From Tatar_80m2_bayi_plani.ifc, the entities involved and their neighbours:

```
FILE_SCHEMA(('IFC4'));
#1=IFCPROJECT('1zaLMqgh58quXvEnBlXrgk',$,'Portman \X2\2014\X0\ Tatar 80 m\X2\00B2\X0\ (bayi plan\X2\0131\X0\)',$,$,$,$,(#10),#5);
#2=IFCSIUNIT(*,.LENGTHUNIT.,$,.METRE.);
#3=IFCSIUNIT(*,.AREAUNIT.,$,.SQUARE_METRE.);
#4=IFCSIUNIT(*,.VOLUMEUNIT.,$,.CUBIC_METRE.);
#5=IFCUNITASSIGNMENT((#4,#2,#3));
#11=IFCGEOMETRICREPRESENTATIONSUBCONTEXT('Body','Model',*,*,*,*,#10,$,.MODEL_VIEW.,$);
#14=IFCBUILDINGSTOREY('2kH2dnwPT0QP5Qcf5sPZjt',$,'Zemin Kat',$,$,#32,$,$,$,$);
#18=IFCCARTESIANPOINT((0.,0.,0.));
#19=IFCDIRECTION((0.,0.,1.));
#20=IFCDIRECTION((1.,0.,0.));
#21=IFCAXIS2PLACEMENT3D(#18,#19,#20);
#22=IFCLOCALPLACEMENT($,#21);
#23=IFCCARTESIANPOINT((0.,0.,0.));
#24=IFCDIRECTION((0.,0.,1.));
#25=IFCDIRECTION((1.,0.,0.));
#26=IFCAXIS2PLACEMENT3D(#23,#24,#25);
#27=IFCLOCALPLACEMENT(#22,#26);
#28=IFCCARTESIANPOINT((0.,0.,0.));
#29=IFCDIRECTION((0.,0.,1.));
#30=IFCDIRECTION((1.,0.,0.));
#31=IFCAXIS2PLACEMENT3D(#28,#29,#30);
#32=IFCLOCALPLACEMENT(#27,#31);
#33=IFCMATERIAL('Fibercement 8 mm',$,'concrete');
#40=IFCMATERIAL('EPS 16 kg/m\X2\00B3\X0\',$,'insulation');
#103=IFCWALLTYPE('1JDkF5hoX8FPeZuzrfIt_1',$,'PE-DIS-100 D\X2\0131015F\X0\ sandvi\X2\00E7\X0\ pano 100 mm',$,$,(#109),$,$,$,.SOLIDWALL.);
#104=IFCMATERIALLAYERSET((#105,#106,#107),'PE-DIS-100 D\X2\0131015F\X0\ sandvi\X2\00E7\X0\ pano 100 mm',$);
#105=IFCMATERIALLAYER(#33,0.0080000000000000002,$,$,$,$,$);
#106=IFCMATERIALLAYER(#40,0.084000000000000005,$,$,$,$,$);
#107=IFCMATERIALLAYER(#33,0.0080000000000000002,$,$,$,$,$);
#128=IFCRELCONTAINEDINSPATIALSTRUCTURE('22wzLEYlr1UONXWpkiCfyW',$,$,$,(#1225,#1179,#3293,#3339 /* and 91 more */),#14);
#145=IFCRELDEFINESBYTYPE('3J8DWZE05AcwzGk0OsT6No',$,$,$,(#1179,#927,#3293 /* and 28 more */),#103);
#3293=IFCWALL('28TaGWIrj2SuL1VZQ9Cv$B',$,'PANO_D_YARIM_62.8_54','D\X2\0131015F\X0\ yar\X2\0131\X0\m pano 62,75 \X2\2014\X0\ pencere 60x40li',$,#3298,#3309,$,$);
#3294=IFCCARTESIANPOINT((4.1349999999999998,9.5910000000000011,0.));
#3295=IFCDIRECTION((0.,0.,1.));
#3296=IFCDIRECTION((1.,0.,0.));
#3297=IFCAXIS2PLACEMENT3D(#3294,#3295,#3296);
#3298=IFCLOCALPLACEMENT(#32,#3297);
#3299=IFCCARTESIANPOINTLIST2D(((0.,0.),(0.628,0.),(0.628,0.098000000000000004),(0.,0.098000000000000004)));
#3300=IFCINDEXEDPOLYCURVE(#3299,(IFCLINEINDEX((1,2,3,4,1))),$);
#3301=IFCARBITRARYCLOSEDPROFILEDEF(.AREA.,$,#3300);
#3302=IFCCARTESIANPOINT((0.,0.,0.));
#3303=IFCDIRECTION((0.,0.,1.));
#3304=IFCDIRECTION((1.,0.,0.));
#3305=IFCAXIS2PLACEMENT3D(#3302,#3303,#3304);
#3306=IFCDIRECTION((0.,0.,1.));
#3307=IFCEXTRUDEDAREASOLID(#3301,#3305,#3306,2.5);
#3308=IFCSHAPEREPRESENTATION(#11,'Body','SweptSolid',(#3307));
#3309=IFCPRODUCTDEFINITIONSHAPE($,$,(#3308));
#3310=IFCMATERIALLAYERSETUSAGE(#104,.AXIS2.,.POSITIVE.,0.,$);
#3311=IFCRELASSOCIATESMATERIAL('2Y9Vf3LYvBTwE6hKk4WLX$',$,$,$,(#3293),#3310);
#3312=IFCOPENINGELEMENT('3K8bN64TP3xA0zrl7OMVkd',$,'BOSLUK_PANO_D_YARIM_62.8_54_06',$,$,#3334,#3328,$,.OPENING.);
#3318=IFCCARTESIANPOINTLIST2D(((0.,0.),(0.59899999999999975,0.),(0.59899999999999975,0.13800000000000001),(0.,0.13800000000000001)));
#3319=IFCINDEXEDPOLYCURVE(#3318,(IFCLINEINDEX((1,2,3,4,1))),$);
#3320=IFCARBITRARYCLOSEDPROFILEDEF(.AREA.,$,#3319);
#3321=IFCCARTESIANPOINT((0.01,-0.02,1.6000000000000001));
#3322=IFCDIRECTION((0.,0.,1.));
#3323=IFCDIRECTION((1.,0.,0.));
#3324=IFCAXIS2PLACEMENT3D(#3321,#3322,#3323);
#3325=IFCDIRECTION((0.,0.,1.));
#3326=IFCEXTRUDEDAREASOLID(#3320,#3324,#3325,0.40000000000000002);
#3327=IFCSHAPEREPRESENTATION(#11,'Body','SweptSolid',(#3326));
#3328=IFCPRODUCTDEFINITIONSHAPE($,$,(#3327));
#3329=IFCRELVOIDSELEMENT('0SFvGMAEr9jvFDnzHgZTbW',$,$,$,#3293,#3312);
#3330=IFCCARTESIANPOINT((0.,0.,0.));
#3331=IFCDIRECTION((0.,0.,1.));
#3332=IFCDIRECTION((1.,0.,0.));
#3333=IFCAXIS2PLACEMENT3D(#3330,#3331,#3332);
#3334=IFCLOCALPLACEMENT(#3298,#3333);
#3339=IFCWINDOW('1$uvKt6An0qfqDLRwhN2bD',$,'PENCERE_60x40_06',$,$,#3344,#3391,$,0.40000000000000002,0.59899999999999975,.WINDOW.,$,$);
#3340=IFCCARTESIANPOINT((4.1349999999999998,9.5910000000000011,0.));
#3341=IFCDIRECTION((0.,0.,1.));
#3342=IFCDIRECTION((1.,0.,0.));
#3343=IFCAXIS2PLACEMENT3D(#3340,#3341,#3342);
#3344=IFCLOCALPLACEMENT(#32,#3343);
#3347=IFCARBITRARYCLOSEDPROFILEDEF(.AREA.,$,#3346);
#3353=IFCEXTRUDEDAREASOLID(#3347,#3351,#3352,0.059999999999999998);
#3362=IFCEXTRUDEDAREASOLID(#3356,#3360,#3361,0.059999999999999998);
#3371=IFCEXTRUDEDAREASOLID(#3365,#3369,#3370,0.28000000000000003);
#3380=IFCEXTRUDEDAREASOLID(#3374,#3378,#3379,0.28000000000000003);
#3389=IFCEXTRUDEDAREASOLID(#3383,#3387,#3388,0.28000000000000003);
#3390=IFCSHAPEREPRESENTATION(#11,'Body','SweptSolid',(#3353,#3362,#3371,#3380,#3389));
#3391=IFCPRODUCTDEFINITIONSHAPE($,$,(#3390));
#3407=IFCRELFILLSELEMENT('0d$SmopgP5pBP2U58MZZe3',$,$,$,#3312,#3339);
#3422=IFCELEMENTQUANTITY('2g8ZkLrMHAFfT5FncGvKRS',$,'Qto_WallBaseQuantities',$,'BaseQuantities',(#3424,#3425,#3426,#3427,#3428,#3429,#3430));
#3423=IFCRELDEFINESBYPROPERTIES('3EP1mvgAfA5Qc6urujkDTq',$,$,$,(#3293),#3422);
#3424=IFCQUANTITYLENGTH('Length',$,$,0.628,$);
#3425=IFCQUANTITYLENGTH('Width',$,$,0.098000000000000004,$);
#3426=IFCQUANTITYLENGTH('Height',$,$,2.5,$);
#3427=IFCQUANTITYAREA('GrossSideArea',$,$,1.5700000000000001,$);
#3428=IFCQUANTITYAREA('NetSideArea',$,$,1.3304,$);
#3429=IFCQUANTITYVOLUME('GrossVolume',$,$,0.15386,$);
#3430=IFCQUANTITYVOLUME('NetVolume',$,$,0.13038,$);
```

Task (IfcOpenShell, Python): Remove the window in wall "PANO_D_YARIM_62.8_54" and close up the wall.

```python
import ifcopenshell
import ifcopenshell.api.feature
import ifcopenshell.api.pset
import ifcopenshell.api.root
import ifcopenshell.geom
import ifcopenshell.util.element
import ifcopenshell.util.shape
import ifcopenshell.util.unit

model = ifcopenshell.open("Tatar_80m2_bayi_plani.ifc")
area_scale = ifcopenshell.util.unit.calculate_unit_scale(model, "AREAUNIT")
volume_scale = ifcopenshell.util.unit.calculate_unit_scale(model, "VOLUMEUNIT")
settings = ifcopenshell.geom.settings()


def volume(element):
    """Net volume in cubic metres, openings subtracted."""
    shape = ifcopenshell.geom.create_shape(settings, element)
    return ifcopenshell.util.shape.get_volume(shape.geometry)


window = model.by_id(3339)
opening = window.FillsVoids[0].RelatingOpeningElement
wall = opening.VoidsElements[0].RelatingBuildingElement
before = volume(wall)

ifcopenshell.api.root.remove_product(model, product=window)
ifcopenshell.api.feature.remove_feature(model, feature=opening)

after = volume(wall)
thickness = 0.098  # wall thickness in metres

# Update the wall's stored quantities.
qto = model.by_id(ifcopenshell.util.element.get_pset(wall, "Qto_WallBaseQuantities", should_inherit=False)["id"])
ifcopenshell.api.pset.edit_qto(model, qto=qto, properties={
    "NetSideArea": after / thickness / area_scale,
    "NetVolume": after / volume_scale,
})

print(f"wall volume {before:.3f} -> {after:.3f} m3")

model.write("Tatar_80m2_bayi_plani_updated.ifc")
```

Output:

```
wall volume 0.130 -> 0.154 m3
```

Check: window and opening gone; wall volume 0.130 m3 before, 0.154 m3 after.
